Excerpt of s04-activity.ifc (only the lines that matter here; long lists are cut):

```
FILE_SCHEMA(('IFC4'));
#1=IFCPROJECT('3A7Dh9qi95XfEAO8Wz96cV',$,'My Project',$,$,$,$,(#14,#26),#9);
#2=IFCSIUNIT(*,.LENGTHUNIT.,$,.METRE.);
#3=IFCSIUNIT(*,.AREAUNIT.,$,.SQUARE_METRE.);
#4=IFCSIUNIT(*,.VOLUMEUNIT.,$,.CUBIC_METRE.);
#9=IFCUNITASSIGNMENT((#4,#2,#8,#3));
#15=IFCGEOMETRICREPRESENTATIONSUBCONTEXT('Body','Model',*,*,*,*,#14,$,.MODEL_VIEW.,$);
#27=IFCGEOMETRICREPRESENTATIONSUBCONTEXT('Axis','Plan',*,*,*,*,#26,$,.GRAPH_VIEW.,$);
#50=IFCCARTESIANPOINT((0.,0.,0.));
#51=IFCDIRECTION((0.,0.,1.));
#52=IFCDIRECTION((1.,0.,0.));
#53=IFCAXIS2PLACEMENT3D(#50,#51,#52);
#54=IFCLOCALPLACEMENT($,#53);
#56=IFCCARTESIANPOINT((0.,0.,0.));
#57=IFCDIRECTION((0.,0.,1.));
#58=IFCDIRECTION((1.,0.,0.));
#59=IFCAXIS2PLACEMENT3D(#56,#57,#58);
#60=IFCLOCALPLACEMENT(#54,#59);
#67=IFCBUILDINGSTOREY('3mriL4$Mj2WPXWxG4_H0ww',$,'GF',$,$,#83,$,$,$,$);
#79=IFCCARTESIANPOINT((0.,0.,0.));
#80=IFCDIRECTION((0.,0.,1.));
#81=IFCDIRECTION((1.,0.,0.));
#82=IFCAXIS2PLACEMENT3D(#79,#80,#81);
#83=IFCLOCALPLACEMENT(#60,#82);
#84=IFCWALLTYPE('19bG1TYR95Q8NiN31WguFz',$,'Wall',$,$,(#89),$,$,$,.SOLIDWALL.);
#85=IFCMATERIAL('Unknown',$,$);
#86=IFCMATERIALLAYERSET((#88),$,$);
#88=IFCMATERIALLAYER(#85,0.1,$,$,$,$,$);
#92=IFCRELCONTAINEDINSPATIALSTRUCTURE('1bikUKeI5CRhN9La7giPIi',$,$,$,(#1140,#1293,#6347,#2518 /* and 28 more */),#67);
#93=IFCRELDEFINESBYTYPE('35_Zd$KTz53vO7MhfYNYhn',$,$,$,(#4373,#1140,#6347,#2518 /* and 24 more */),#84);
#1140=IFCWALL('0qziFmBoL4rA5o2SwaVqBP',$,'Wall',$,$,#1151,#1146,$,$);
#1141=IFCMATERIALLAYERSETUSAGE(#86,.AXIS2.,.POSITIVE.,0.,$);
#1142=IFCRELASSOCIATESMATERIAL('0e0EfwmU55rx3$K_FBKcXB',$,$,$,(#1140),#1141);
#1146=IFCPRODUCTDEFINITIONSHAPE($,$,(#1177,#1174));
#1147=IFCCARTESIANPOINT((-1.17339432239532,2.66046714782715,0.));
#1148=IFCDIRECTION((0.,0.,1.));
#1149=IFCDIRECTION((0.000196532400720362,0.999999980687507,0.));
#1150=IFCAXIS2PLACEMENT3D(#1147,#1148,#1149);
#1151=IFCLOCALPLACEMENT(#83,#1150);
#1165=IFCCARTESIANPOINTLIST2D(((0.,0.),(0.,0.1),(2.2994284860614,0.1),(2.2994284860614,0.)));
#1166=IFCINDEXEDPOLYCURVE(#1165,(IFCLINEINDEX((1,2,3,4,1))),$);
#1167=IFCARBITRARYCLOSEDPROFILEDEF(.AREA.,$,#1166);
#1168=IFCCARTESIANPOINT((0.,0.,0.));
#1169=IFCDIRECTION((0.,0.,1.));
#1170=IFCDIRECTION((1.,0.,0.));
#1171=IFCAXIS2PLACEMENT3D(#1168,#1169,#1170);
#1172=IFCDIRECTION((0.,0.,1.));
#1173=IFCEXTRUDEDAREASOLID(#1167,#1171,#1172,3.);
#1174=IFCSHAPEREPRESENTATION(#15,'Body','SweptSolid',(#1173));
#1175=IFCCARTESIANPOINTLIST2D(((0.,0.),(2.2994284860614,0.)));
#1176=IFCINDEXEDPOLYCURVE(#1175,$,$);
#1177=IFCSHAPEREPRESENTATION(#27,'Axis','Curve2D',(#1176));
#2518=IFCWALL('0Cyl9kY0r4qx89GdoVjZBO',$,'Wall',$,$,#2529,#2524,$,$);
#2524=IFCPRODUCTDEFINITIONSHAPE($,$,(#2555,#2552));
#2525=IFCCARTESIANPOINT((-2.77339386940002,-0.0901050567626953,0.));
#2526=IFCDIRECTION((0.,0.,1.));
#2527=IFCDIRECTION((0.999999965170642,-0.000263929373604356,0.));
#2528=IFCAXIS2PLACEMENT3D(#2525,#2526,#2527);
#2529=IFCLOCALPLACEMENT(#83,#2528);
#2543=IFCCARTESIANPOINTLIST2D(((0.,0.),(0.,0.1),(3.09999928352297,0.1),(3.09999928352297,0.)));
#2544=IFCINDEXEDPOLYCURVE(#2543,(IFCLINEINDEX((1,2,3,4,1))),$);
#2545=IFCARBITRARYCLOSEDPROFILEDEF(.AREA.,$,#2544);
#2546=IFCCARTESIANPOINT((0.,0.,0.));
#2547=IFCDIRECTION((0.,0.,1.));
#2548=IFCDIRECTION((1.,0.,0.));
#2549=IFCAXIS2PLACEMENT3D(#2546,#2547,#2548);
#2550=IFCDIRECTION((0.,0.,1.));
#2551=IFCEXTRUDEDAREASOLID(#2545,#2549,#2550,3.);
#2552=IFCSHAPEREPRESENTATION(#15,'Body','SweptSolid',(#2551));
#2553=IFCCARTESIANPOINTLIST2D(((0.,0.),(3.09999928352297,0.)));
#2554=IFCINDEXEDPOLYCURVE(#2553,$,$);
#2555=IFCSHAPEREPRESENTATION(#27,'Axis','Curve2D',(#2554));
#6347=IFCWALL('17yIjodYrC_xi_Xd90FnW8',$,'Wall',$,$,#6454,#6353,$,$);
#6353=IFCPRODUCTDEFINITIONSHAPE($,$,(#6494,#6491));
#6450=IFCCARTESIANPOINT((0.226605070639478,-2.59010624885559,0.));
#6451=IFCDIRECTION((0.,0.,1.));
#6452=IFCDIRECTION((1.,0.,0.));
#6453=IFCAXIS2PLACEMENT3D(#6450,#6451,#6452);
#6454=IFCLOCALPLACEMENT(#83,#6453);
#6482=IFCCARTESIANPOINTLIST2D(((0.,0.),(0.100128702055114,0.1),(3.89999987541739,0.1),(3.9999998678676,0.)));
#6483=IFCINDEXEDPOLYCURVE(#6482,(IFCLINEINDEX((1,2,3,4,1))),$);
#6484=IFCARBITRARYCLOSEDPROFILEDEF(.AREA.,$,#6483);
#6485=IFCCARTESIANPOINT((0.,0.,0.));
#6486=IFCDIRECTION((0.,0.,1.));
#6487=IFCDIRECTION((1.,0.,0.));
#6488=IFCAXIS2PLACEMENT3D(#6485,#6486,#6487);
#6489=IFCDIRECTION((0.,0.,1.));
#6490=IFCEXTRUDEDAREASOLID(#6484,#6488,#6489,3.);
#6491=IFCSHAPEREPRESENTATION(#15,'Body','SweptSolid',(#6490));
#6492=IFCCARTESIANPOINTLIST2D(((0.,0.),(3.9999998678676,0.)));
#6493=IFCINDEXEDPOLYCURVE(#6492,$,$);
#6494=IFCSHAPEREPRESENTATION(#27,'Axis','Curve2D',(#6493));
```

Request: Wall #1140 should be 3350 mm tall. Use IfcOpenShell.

```python
import ifcopenshell
import ifcopenshell.geom
import ifcopenshell.util.representation
import ifcopenshell.util.shape
import ifcopenshell.util.unit

model = ifcopenshell.open("s04-activity.ifc")
unit_scale = ifcopenshell.util.unit.calculate_unit_scale(model)
settings = ifcopenshell.geom.settings()


def volume(element):
    """Net volume in cubic metres, openings subtracted."""
    shape = ifcopenshell.geom.create_shape(settings, element)
    return ifcopenshell.util.shape.get_volume(shape.geometry)


wall = model.by_id(1140)
before = volume(wall)

body = ifcopenshell.util.representation.get_representation(wall, "Model", "Body")
solid = body.Items[0]
old_height = solid.Depth
solid.Depth = 3.35 / unit_scale
after = volume(wall)

print(f"height {old_height:g} -> {solid.Depth:g}, volume {before:.3f} -> {after:.3f} m3")

model.write("s04-activity_updated.ifc")
```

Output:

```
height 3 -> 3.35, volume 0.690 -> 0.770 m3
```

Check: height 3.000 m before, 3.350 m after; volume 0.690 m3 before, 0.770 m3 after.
